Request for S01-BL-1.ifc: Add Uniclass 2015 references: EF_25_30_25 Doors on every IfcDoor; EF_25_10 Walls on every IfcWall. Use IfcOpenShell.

First a look at what the model holds.

```python
import ifcopenshell

model = ifcopenshell.open("S01-BL-1.ifc")
print(model.schema)
print("classifications:", [c.Name for c in model.by_type("IfcClassification")])
for ifc_class in ("IfcDoor", "IfcRoof", "IfcStair", "IfcWall", "IfcWindow"):
    print(ifc_class, len(model.by_type(ifc_class)))
```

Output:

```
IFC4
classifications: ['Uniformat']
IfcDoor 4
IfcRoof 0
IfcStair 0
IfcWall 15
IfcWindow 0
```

```python
import ifcopenshell
import ifcopenshell.api.classification

model = ifcopenshell.open("S01-BL-1.ifc")

system = ifcopenshell.api.classification.add_classification(model, classification="Uniclass 2015")

codes = {
    "IfcDoor": ("EF_25_30_25", "Doors"),
    "IfcWall": ("EF_25_10", "Walls"),
}
for ifc_class, (code, name) in codes.items():
    products = model.by_type(ifc_class)
    ifcopenshell.api.classification.add_reference(
        model, products=products, classification=system, identification=code, name=name
    )
    print(code, len(products))

model.write("S01-BL-1_rev.ifc")
```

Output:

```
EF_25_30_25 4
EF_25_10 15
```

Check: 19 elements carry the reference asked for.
